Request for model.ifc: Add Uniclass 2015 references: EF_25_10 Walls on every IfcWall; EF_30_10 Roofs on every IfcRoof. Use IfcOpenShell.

First a look at what the model holds.

```python
import ifcopenshell

model = ifcopenshell.open("model.ifc")
print(model.schema)
print("classifications:", [c.Name for c in model.by_type("IfcClassification")])
for ifc_class in ("IfcDoor", "IfcRoof", "IfcStair", "IfcWall", "IfcWindow"):
    print(ifc_class, len(model.by_type(ifc_class)))
```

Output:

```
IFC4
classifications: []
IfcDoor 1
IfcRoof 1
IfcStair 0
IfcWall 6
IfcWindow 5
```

```python
import ifcopenshell
import ifcopenshell.api.classification

model = ifcopenshell.open("model.ifc")

system = ifcopenshell.api.classification.add_classification(model, classification="Uniclass 2015")

codes = {
    "IfcWall": ("EF_25_10", "Walls"),
    "IfcRoof": ("EF_30_10", "Roofs"),
}
for ifc_class, (code, name) in codes.items():
    products = model.by_type(ifc_class)
    ifcopenshell.api.classification.add_reference(
        model, products=products, classification=system, identification=code, name=name
    )
    print(code, len(products))

model.write("model_rev.ifc")
```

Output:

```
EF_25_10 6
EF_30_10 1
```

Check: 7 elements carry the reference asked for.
